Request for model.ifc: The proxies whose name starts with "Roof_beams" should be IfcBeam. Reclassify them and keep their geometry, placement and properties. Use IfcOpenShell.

First a look at what the model holds.

```python
import re

import ifcopenshell

model = ifcopenshell.open("model.ifc")
print(model.schema)
seen = {}
for e in model.by_type("IfcBuildingElementProxy"):
    name = re.sub(r":\d+(:\d+)?$", "", e.Name or "")  # drop the element id that some exporters append
    seen[name] = seen.get(name, 0) + 1
for name, count in sorted(seen.items()):
    print(count, "x", name)
```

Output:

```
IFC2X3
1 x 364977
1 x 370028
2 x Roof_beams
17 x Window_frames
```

```python
import ifcopenshell
import ifcopenshell.api.root

model = ifcopenshell.open("model.ifc")

proxies = [e.id() for e in model.by_type("IfcBuildingElementProxy") if (e.Name or "").startswith("Roof_beams")]
for step_id in proxies:
    proxy = model.by_id(step_id)
    # Reclassifying a typed element also reclassifies its type and the type's other occurrences.
    if proxy.is_a("IfcBuildingElementProxy"):
        ifcopenshell.api.root.reassign_class(model, product=proxy, ifc_class="IfcBeam")

print(sum(model.by_id(i).is_a("IfcBeam") for i in proxies), "reclassified")

model.write("model_v2.ifc")
```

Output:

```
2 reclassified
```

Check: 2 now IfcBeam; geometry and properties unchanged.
